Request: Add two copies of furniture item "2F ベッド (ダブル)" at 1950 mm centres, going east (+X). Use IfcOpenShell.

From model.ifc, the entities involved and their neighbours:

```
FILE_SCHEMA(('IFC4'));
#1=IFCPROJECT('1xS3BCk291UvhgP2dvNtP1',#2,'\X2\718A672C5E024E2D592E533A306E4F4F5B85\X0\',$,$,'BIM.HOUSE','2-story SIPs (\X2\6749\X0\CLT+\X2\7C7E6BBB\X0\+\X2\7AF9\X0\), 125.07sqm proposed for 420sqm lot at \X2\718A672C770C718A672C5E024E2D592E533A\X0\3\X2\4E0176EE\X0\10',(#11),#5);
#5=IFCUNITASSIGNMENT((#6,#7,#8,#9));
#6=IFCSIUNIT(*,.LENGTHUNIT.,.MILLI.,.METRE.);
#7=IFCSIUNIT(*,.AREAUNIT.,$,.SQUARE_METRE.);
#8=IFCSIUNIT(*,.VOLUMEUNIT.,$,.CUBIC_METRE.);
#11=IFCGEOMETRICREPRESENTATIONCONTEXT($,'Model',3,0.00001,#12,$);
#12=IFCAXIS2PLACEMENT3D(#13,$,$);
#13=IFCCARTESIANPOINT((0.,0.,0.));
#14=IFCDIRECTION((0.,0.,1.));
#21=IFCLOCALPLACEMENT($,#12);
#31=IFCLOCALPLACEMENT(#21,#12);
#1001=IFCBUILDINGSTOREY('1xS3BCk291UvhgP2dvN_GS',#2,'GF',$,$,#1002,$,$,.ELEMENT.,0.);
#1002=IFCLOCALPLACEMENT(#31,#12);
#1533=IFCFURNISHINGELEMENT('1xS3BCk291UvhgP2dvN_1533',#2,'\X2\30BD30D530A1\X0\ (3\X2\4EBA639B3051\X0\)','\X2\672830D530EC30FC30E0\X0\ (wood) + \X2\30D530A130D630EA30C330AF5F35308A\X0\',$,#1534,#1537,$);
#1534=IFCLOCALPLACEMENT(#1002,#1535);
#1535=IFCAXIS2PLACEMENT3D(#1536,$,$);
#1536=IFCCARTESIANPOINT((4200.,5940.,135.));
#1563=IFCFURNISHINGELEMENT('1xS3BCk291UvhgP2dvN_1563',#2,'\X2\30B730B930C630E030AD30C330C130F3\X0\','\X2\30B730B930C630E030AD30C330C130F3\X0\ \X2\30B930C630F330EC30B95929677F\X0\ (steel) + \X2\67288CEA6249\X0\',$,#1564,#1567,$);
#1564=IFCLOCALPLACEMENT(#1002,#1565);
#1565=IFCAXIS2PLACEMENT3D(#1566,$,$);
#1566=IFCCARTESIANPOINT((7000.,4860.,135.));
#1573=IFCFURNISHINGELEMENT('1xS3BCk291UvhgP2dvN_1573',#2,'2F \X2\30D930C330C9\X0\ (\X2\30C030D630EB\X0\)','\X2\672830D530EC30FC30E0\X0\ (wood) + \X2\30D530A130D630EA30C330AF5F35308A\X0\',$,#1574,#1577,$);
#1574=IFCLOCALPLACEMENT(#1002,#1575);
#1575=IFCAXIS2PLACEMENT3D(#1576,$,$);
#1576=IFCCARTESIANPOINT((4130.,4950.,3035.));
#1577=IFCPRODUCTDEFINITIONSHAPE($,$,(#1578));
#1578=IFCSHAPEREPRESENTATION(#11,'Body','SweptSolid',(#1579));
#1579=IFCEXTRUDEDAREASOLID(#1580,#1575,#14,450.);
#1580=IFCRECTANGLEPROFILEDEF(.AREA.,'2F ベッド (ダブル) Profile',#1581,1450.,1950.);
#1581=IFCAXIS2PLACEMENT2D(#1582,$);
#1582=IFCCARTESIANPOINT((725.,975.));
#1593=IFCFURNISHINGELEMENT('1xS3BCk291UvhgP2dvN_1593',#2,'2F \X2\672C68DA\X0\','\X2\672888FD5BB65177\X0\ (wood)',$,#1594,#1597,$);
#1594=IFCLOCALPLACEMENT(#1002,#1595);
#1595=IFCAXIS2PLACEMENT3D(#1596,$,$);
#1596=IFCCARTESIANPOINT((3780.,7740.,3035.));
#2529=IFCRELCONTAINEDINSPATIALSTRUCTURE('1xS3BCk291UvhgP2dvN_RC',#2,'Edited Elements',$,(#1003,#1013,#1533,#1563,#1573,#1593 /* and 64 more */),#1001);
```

```python
import numpy as np
import ifcopenshell
import ifcopenshell.api.geometry
import ifcopenshell.api.root
import ifcopenshell.util.element
import ifcopenshell.util.placement

model = ifcopenshell.open("model.ifc")


def reuse_history(source, copy):
    """copy_class also copies each property set's owner history, people and application; keep the originals."""
    for rel in copy.IsDefinedBy:
        if rel.is_a("IfcRelDefinesByProperties") and (history := rel.RelatingPropertyDefinition.OwnerHistory):
            rel.RelatingPropertyDefinition.OwnerHistory = source.OwnerHistory
            ifcopenshell.util.element.remove_deep2(model, history)


source = model.by_id(1573)
base = ifcopenshell.util.placement.get_local_placement(source.ObjectPlacement)
step = np.array([1.0, 0.0, 0.0]) * 1950.0

for i in range(1, 3):
    copy = ifcopenshell.api.root.copy_class(model, product=source)
    copy.Representation = ifcopenshell.util.element.copy_deep(
        model, source.Representation, exclude=["IfcGeometricRepresentationContext", "IfcRepresentationMap"]
    )
    reuse_history(source, copy)
    matrix = base.copy()
    matrix[:3, 3] += i * step
    print("added at", matrix[:3, 3].round(3) + 0.0)
    ifcopenshell.api.geometry.edit_object_placement(model, product=copy, matrix=matrix, is_si=False)

model.write("model_updated.ifc")
```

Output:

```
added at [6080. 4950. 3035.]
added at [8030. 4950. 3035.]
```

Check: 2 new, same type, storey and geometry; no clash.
